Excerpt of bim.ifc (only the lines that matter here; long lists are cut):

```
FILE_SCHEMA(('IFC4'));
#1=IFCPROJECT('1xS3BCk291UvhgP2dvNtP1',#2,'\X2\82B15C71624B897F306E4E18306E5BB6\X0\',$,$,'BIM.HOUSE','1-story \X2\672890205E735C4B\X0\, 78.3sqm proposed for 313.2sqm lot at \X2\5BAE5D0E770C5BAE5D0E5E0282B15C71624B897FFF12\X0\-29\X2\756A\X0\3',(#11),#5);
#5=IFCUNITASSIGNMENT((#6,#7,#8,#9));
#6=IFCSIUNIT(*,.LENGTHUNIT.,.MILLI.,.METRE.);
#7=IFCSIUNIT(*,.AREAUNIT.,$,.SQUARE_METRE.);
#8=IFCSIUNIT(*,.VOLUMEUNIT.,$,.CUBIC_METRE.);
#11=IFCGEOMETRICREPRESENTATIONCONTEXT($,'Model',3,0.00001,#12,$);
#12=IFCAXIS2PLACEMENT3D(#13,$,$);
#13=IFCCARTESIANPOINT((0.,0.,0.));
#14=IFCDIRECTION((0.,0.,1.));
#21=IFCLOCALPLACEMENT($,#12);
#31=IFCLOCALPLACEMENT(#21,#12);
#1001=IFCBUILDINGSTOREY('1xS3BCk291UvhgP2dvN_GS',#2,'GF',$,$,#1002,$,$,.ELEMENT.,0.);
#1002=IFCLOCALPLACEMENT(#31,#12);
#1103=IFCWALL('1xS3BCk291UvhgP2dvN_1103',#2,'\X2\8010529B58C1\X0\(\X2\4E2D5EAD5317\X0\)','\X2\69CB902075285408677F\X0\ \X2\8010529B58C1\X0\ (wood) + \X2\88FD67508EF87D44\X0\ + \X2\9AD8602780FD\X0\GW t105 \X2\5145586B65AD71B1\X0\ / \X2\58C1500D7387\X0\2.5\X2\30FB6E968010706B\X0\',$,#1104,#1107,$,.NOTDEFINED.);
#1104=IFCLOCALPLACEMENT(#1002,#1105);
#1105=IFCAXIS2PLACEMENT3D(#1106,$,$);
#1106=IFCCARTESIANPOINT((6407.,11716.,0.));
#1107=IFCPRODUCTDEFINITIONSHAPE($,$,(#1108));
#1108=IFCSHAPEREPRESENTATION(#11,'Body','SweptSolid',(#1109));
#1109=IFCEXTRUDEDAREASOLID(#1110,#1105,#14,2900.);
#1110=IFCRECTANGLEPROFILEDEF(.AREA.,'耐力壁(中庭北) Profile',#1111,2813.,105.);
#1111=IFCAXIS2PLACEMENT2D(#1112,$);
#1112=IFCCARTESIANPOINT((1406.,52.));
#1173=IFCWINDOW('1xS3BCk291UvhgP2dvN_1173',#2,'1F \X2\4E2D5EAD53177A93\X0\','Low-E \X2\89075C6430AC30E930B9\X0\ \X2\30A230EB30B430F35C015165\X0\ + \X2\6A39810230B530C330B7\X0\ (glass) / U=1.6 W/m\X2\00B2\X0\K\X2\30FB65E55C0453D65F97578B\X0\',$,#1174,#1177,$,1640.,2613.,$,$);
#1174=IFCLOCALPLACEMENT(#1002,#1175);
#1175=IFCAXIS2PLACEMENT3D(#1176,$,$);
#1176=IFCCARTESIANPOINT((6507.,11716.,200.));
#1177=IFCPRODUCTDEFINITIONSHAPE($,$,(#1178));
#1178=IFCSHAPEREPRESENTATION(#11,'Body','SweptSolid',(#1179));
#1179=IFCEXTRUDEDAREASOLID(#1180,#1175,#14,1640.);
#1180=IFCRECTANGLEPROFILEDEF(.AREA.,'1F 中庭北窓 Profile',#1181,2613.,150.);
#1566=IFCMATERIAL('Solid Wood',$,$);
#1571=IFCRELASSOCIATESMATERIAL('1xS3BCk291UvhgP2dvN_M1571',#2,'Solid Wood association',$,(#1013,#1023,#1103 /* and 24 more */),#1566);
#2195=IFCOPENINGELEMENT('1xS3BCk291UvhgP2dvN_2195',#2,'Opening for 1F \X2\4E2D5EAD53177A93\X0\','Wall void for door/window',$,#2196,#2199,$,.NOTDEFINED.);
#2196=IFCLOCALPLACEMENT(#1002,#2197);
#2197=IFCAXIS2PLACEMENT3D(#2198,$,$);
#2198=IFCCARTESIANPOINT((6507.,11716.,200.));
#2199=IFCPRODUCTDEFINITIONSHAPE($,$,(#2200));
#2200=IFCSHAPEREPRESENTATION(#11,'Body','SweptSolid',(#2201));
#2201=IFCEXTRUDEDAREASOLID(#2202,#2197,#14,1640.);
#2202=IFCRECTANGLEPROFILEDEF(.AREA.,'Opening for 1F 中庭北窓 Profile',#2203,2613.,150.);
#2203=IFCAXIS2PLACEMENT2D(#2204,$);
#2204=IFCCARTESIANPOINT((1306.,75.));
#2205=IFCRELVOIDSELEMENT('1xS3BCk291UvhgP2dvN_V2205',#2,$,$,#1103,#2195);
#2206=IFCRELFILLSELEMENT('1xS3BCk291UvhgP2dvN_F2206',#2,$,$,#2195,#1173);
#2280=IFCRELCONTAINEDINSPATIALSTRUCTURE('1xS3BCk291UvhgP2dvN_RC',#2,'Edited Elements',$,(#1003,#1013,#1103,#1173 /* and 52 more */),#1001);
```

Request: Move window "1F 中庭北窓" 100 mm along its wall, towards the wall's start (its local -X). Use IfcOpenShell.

```python
import ifcopenshell
import ifcopenshell.api.geometry
import ifcopenshell.util.placement
import ifcopenshell.util.unit

model = ifcopenshell.open("bim.ifc")
unit_scale = ifcopenshell.util.unit.calculate_unit_scale(model)

window = model.by_guid("1xS3BCk291UvhgP2dvN_1173")
opening = window.FillsVoids[0].RelatingOpeningElement
wall = opening.VoidsElements[0].RelatingBuildingElement

wall_matrix = ifcopenshell.util.placement.get_local_placement(wall.ObjectPlacement)
shift = wall_matrix[:3, 0] * -0.1 / unit_scale
before = ifcopenshell.util.placement.get_local_placement(window.ObjectPlacement)[:3, 3].copy()

# The window is not placed relative to its opening, so move both.
for product in (opening, window):
    matrix = ifcopenshell.util.placement.get_local_placement(product.ObjectPlacement)
    matrix[:3, 3] += shift
    ifcopenshell.api.geometry.edit_object_placement(model, product=product, matrix=matrix, is_si=False)

after = ifcopenshell.util.placement.get_local_placement(window.ObjectPlacement)[:3, 3]
print("window moved by", (after - before).round(3) + 0.0)

model.write("bim_v2.ifc")
```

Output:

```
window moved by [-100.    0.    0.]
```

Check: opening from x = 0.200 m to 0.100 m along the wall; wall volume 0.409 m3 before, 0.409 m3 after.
